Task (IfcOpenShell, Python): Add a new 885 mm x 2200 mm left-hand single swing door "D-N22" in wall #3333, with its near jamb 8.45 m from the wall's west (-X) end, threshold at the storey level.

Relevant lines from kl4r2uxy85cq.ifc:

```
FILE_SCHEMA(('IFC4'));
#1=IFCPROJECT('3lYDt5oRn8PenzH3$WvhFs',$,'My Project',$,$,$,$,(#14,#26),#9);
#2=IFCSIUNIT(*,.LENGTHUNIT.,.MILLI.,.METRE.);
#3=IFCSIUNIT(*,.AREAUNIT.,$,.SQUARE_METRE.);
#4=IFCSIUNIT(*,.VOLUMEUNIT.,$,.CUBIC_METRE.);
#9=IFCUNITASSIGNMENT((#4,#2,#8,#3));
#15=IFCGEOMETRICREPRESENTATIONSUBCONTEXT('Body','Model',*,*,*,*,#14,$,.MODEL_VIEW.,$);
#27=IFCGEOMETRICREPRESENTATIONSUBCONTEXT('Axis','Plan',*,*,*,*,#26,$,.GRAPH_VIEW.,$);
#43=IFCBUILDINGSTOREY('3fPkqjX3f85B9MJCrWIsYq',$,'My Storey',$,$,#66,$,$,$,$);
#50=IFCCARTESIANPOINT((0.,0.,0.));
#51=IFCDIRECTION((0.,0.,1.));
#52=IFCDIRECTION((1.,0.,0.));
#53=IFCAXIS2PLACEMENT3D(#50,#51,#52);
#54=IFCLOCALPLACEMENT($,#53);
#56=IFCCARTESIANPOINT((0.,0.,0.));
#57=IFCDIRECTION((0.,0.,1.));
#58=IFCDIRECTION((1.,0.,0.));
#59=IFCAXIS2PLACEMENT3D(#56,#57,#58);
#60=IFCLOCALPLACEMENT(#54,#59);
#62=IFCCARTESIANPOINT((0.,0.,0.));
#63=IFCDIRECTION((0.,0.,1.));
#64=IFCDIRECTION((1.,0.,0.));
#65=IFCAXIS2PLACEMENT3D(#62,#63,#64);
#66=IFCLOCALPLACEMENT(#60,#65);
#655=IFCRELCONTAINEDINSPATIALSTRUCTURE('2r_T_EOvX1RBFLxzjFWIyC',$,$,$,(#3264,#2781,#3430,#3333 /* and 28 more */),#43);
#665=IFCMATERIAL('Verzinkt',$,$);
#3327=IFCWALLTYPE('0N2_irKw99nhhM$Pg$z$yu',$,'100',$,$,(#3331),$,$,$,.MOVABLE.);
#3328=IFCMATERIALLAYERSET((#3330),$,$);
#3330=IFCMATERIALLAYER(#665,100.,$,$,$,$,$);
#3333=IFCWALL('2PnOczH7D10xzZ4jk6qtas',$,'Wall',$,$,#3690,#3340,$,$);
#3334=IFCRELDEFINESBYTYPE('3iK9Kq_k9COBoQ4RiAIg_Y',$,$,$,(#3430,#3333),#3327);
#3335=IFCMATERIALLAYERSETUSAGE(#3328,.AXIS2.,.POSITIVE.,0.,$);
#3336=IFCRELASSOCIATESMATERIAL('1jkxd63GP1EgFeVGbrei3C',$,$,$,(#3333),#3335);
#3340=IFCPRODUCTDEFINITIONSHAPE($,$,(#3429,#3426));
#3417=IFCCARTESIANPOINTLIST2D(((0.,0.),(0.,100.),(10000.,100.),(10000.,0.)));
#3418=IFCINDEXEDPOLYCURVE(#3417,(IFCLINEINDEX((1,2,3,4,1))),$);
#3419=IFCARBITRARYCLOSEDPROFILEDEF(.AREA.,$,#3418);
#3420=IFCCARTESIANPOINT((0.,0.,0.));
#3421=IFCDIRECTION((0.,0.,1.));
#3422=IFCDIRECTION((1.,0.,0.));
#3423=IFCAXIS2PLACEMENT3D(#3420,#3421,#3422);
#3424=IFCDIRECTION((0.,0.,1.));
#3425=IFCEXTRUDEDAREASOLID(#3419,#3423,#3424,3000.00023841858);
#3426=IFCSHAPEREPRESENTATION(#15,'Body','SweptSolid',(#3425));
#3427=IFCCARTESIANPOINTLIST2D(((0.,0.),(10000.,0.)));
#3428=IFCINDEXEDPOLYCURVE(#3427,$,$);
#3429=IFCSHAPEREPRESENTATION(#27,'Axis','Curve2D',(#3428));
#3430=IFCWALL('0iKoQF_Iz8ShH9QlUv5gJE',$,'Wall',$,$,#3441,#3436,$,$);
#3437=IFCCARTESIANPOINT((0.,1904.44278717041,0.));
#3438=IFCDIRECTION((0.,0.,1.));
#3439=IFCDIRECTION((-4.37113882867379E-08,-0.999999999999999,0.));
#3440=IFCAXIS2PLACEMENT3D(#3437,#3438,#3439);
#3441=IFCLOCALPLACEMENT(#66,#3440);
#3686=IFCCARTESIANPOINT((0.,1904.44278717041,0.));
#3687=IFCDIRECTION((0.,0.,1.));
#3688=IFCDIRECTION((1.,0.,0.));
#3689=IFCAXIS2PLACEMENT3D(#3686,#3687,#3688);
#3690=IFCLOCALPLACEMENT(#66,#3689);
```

```python
import numpy as np
import ifcopenshell
import ifcopenshell.api.feature
import ifcopenshell.api.geometry
import ifcopenshell.api.root
import ifcopenshell.api.spatial
import ifcopenshell.geom
import ifcopenshell.util.element
import ifcopenshell.util.placement
import ifcopenshell.util.representation
import ifcopenshell.util.shape
import ifcopenshell.util.unit

model = ifcopenshell.open("kl4r2uxy85cq.ifc")
unit_scale = ifcopenshell.util.unit.calculate_unit_scale(model)
settings = ifcopenshell.geom.settings()


def volume(element):
    """Net volume in cubic metres, openings subtracted."""
    shape = ifcopenshell.geom.create_shape(settings, element)
    return ifcopenshell.util.shape.get_volume(shape.geometry)


wall = model.by_guid("2PnOczH7D10xzZ4jk6qtas")
storey = ifcopenshell.util.element.get_container(wall, ifc_class="IfcBuildingStorey")
context = ifcopenshell.util.representation.get_context(model, "Model", "Body", "MODEL_VIEW")
before = volume(wall)

width, height, from_end, sill = 0.885, 2.2, 8.45, 0.0  # metres

# The wall runs along its own X axis, and the end named is its -X end.
wall_shape = ifcopenshell.geom.create_shape(settings, wall)
x, y, z = ifcopenshell.util.shape.get_vertices(wall_shape.geometry).T
start = x.min() + from_end
face, thickness = float(y.min()), float(y.max() - y.min())
wall_matrix = ifcopenshell.util.placement.get_local_placement(wall.ObjectPlacement)
level = ifcopenshell.util.placement.get_local_placement(storey.ObjectPlacement)[2, 3]


def in_wall(x, y):
    """Placement at x, y metres in the wall's axes, at sill height."""
    matrix = wall_matrix.copy()
    matrix[:, 3] = wall_matrix @ np.array([x / unit_scale, y / unit_scale, 0.0, 1.0])
    matrix[2, 3] = level + sill / unit_scale
    return matrix


# Opening: a box that overshoots both wall faces by 50 mm.
opening = ifcopenshell.api.root.create_entity(model, ifc_class="IfcOpeningElement", predefined_type="OPENING")
box = ifcopenshell.api.geometry.add_wall_representation(
    model, context=context, length=width, height=height, thickness=thickness + 0.1
)
ifcopenshell.api.geometry.assign_representation(model, product=opening, representation=box)
ifcopenshell.api.geometry.edit_object_placement(model, product=opening, matrix=in_wall(start, face - 0.05), is_si=False)
ifcopenshell.api.feature.add_feature(model, feature=opening, element=wall)

door = ifcopenshell.api.root.create_entity(model, ifc_class="IfcDoor", name="D-N22", predefined_type="DOOR")
door.OverallWidth, door.OverallHeight = width / unit_scale, height / unit_scale
door.OperationType = "SINGLE_SWING_LEFT"
body = ifcopenshell.api.geometry.add_door_representation(
    model,
    context=context,
    overall_width=door.OverallWidth,
    overall_height=door.OverallHeight,
    operation_type="SINGLE_SWING_LEFT",
    lining_properties={"LiningDepth": thickness / unit_scale, "ThresholdDepth": thickness / unit_scale},
)
ifcopenshell.api.geometry.assign_representation(model, product=door, representation=body)
ifcopenshell.api.spatial.assign_container(model, products=[door], relating_structure=storey)
ifcopenshell.api.feature.add_filling(model, opening=opening, element=door)

# The lining spans the wall, so the door starts at the wall face.
ifcopenshell.api.geometry.edit_object_placement(model, product=door, matrix=in_wall(start, face), is_si=False)

after = volume(wall)

print(f"wall volume {before:.3f} -> {after:.3f} m3")

model.write("kl4r2uxy85cq_updated.ifc")
```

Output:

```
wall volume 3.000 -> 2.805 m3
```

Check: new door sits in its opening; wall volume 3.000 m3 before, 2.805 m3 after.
